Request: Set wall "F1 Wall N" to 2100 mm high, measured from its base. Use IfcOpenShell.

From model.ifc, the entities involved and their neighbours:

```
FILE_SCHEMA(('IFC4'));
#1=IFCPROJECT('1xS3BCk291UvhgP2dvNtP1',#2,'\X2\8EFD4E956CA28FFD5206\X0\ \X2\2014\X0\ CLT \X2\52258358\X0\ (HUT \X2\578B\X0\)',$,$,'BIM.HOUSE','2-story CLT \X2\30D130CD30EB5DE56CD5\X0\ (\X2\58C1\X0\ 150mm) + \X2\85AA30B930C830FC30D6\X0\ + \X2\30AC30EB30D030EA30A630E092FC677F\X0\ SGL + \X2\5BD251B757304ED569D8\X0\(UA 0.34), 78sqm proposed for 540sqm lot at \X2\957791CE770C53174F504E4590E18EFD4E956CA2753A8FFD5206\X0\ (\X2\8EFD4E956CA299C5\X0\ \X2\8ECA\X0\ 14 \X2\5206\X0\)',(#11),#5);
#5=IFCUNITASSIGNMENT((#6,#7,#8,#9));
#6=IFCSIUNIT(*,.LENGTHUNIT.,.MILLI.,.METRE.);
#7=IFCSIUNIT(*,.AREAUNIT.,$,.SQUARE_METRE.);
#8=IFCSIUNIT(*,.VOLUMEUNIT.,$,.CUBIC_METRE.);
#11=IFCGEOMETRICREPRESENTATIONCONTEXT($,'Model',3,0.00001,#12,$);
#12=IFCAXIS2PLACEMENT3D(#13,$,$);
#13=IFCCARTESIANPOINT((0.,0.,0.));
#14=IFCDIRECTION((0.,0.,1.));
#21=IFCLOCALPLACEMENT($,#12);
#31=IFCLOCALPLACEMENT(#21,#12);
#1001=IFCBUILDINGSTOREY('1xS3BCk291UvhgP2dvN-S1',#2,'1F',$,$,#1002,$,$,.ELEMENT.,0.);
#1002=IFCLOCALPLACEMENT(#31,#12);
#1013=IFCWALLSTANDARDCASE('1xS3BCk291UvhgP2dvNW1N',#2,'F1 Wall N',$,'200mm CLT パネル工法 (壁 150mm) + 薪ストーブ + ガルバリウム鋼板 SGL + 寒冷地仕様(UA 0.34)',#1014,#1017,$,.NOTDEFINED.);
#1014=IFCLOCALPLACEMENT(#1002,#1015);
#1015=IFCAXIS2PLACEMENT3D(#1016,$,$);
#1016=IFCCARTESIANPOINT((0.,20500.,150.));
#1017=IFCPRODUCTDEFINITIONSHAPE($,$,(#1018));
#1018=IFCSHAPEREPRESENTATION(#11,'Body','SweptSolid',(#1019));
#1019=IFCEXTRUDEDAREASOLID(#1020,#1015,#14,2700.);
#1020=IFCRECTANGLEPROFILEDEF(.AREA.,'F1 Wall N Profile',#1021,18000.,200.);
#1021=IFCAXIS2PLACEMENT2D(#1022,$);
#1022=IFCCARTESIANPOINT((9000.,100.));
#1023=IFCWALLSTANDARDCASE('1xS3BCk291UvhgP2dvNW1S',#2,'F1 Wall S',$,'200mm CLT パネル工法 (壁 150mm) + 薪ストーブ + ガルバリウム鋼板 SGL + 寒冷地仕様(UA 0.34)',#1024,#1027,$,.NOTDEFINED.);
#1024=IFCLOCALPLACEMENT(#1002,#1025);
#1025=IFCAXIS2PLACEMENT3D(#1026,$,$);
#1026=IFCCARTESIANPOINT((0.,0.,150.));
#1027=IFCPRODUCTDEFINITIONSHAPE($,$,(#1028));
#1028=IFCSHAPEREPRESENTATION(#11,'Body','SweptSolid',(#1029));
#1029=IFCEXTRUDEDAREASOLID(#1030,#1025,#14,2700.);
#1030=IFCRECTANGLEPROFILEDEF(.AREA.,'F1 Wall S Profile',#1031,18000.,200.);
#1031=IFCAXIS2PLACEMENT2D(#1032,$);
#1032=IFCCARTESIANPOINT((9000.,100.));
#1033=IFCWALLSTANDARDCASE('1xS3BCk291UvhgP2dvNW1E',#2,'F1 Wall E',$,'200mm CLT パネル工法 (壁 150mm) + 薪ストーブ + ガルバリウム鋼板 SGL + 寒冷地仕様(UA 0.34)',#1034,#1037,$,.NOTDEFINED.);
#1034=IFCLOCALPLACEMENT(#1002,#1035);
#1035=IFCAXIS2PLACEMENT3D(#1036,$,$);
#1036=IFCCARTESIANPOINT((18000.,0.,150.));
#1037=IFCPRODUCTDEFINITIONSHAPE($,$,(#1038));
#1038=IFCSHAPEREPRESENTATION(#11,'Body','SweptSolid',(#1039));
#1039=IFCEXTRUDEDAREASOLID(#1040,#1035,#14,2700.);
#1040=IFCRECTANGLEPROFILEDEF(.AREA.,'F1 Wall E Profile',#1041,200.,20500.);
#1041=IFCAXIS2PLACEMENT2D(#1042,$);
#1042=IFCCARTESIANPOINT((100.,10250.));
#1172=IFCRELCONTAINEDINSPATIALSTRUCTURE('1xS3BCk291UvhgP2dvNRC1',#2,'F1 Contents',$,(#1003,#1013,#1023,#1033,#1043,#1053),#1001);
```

```python
import ifcopenshell
import ifcopenshell.geom
import ifcopenshell.util.shape

model = ifcopenshell.open("model.ifc")
settings = ifcopenshell.geom.settings()


def volume(element):
    """Net volume in cubic metres, openings subtracted."""
    shape = ifcopenshell.geom.create_shape(settings, element)
    return ifcopenshell.util.shape.get_volume(shape.geometry)


wall = model.by_id(1013)
before = volume(wall)

body = next(r for r in wall.Representation.Representations if r.RepresentationIdentifier == "Body")
solid = body.Items[0]
old_height = solid.Depth
solid.Depth = 2100.0
after = volume(wall)

print(f"height {old_height:g} -> {solid.Depth:g}, volume {before:.3f} -> {after:.3f} m3")

model.write("model-out.ifc")
```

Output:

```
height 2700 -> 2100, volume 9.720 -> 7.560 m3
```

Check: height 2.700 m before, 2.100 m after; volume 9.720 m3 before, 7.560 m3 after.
